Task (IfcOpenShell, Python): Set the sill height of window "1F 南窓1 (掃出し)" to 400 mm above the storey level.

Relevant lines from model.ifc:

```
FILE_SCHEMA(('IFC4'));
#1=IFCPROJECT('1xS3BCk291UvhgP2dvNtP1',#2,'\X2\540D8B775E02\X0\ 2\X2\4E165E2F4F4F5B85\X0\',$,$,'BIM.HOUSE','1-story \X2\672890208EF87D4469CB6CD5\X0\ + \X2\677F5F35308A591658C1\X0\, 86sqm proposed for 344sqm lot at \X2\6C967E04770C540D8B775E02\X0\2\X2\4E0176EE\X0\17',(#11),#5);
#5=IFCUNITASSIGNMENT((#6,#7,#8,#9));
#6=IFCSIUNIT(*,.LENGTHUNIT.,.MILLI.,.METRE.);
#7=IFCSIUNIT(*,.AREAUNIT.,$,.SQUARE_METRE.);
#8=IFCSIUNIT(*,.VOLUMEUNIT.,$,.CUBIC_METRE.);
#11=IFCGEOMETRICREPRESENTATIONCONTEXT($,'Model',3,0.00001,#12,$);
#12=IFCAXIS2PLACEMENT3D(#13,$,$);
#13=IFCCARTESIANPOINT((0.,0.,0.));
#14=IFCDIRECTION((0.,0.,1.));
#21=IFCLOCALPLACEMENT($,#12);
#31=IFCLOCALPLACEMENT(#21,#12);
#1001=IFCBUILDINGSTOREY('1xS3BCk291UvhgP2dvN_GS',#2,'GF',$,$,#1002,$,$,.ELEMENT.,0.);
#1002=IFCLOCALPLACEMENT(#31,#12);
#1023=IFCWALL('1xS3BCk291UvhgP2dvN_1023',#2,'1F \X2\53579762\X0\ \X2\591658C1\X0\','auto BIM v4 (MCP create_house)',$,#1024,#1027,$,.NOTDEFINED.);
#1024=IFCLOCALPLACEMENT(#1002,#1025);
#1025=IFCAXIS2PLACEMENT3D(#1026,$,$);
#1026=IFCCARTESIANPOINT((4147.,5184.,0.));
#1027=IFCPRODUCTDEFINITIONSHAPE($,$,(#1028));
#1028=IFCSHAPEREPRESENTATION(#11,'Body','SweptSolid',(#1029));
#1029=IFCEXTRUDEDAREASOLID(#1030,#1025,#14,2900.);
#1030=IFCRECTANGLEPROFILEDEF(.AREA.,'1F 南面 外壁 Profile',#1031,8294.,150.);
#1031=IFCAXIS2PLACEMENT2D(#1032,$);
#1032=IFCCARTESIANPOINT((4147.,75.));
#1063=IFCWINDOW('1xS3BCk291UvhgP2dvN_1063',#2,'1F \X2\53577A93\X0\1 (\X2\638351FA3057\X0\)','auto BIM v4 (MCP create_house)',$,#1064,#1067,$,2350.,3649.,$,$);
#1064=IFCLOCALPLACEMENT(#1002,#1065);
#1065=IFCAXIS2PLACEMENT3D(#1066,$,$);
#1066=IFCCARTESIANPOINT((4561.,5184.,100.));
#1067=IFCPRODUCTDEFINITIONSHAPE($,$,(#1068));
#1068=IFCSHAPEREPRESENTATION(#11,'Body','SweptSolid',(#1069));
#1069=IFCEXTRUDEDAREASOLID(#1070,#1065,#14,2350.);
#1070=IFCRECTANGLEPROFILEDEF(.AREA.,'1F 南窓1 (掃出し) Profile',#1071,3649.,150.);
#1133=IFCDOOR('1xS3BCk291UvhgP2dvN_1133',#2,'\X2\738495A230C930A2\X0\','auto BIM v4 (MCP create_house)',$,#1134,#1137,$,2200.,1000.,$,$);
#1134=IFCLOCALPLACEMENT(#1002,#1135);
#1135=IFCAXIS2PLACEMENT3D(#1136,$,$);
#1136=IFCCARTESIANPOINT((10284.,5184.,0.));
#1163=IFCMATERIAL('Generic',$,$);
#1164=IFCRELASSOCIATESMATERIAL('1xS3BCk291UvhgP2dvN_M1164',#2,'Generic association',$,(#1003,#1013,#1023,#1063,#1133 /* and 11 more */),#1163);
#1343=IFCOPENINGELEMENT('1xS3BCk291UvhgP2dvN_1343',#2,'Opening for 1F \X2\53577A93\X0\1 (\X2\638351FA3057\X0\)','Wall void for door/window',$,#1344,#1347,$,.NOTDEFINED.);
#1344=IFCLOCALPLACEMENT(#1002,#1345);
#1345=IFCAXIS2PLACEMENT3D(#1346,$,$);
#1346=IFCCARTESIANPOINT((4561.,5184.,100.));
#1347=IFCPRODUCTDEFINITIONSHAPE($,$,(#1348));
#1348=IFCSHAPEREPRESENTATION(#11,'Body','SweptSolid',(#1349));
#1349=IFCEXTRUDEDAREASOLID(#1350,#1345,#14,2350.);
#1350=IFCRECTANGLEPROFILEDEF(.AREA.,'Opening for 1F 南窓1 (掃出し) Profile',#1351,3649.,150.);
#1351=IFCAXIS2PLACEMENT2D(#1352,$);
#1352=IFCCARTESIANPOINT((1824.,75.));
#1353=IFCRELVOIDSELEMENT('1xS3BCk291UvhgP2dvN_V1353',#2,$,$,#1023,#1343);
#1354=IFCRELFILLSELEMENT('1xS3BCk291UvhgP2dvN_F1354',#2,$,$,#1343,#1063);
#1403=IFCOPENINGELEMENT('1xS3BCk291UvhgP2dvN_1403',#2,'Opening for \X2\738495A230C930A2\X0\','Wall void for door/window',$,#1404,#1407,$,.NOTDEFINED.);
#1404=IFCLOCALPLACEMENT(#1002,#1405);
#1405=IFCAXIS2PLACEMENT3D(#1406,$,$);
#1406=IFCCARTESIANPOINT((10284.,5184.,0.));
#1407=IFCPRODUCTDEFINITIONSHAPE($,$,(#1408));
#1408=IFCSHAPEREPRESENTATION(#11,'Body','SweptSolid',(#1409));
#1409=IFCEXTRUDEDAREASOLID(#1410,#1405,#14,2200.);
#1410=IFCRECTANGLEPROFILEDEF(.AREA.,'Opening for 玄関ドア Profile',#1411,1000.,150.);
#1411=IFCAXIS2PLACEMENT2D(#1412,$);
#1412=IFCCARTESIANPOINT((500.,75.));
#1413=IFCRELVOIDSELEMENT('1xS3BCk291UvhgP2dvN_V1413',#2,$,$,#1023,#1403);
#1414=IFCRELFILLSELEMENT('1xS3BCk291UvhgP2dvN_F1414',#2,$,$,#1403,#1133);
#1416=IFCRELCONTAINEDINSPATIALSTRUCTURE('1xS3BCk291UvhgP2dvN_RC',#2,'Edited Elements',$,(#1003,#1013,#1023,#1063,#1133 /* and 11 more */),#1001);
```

```python
import numpy as np
import ifcopenshell
import ifcopenshell.api.geometry
import ifcopenshell.geom
import ifcopenshell.util.element
import ifcopenshell.util.placement
import ifcopenshell.util.shape
import ifcopenshell.util.unit

model = ifcopenshell.open("model.ifc")
unit_scale = ifcopenshell.util.unit.calculate_unit_scale(model)

window = model.by_guid("1xS3BCk291UvhgP2dvN_1063")
opening = window.FillsVoids[0].RelatingOpeningElement
storey = ifcopenshell.util.element.get_container(window, ifc_class="IfcBuildingStorey")
level = ifcopenshell.util.placement.get_local_placement(storey.ObjectPlacement)[2, 3]

# The opening's origin need not be at the sill, so measure its lowest point.
shape = ifcopenshell.geom.create_shape(ifcopenshell.geom.settings(), opening)
bottom = ifcopenshell.util.shape.get_shape_bottom_elevation(shape, shape.geometry) / unit_scale
dz = level + 0.4 / unit_scale - bottom

shift = np.array([0.0, 0.0, dz])
# The window is not placed relative to its opening, so move both.
for product in (opening, window):
    matrix = ifcopenshell.util.placement.get_local_placement(product.ObjectPlacement)
    matrix[:3, 3] += shift
    ifcopenshell.api.geometry.edit_object_placement(model, product=product, matrix=matrix, is_si=False)

print(f"moved by {dz * unit_scale:+.3f} m")

model.write("model_v2.ifc")
```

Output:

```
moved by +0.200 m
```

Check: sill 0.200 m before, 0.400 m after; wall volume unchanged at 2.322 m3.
